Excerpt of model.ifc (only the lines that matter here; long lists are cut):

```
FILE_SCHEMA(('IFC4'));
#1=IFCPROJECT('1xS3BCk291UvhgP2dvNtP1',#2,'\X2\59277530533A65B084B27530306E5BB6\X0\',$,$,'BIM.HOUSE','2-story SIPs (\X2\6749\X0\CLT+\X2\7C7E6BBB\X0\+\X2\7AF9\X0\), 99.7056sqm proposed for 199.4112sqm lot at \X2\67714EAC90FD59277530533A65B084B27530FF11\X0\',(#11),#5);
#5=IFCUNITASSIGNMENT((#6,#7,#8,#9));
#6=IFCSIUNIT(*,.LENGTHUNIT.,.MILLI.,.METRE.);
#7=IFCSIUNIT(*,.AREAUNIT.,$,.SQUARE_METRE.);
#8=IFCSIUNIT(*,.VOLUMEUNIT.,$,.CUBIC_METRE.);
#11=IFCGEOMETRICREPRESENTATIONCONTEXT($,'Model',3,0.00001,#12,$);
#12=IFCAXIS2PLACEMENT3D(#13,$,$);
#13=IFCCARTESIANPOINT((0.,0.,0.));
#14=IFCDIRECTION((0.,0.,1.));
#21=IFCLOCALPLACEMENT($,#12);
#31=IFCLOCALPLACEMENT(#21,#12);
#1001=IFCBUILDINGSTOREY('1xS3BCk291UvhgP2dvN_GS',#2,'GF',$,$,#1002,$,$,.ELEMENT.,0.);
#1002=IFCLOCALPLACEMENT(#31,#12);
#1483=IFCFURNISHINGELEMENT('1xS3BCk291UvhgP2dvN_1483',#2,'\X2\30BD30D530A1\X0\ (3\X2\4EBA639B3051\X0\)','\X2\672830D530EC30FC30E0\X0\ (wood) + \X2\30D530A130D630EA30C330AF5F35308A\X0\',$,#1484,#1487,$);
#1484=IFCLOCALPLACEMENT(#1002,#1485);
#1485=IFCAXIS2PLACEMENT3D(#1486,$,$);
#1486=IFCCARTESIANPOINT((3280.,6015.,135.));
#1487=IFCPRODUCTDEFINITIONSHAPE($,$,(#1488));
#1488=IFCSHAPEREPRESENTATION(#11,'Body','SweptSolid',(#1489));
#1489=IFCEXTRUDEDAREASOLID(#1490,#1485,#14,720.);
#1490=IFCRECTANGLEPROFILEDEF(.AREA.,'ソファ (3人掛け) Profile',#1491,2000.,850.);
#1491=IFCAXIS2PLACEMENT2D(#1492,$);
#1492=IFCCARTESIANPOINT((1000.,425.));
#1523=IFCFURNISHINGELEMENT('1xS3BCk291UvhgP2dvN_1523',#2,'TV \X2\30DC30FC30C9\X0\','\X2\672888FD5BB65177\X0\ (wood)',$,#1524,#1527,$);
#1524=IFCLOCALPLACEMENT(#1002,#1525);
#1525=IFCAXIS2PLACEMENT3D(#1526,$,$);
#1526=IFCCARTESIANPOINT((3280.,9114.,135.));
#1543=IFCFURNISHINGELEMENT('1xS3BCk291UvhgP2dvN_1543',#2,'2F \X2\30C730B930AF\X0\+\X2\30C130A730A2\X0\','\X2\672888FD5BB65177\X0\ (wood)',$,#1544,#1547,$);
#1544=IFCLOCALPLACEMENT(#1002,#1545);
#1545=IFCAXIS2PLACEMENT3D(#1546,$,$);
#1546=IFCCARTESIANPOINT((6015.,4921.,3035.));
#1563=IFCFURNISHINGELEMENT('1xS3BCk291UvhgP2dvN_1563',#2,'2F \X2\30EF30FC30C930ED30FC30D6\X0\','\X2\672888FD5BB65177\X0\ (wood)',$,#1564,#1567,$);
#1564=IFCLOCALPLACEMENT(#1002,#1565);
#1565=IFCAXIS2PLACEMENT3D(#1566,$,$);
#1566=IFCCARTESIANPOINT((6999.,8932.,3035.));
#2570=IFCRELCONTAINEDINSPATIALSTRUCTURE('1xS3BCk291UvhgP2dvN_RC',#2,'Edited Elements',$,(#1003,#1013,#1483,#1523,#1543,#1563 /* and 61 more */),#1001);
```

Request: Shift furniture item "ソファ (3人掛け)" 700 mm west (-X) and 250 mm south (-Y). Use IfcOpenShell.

```python
import ifcopenshell
import ifcopenshell.api.geometry
import ifcopenshell.util.placement
import ifcopenshell.util.unit

model = ifcopenshell.open("model.ifc")
unit_scale = ifcopenshell.util.unit.calculate_unit_scale(model)

item = model.by_guid("1xS3BCk291UvhgP2dvN_1483")
matrix = ifcopenshell.util.placement.get_local_placement(item.ObjectPlacement)
matrix[0, 3] -= 0.7 / unit_scale
matrix[1, 3] -= 0.25 / unit_scale
ifcopenshell.api.geometry.edit_object_placement(model, product=item, matrix=matrix, is_si=False)

print(ifcopenshell.util.placement.get_local_placement(item.ObjectPlacement).round(3) + 0.0)

model.write("model_edited.ifc")
```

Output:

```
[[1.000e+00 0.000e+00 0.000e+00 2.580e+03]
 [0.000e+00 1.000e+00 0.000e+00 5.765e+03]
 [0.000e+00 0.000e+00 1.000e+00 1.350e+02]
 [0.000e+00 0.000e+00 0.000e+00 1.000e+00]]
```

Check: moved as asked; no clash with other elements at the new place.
